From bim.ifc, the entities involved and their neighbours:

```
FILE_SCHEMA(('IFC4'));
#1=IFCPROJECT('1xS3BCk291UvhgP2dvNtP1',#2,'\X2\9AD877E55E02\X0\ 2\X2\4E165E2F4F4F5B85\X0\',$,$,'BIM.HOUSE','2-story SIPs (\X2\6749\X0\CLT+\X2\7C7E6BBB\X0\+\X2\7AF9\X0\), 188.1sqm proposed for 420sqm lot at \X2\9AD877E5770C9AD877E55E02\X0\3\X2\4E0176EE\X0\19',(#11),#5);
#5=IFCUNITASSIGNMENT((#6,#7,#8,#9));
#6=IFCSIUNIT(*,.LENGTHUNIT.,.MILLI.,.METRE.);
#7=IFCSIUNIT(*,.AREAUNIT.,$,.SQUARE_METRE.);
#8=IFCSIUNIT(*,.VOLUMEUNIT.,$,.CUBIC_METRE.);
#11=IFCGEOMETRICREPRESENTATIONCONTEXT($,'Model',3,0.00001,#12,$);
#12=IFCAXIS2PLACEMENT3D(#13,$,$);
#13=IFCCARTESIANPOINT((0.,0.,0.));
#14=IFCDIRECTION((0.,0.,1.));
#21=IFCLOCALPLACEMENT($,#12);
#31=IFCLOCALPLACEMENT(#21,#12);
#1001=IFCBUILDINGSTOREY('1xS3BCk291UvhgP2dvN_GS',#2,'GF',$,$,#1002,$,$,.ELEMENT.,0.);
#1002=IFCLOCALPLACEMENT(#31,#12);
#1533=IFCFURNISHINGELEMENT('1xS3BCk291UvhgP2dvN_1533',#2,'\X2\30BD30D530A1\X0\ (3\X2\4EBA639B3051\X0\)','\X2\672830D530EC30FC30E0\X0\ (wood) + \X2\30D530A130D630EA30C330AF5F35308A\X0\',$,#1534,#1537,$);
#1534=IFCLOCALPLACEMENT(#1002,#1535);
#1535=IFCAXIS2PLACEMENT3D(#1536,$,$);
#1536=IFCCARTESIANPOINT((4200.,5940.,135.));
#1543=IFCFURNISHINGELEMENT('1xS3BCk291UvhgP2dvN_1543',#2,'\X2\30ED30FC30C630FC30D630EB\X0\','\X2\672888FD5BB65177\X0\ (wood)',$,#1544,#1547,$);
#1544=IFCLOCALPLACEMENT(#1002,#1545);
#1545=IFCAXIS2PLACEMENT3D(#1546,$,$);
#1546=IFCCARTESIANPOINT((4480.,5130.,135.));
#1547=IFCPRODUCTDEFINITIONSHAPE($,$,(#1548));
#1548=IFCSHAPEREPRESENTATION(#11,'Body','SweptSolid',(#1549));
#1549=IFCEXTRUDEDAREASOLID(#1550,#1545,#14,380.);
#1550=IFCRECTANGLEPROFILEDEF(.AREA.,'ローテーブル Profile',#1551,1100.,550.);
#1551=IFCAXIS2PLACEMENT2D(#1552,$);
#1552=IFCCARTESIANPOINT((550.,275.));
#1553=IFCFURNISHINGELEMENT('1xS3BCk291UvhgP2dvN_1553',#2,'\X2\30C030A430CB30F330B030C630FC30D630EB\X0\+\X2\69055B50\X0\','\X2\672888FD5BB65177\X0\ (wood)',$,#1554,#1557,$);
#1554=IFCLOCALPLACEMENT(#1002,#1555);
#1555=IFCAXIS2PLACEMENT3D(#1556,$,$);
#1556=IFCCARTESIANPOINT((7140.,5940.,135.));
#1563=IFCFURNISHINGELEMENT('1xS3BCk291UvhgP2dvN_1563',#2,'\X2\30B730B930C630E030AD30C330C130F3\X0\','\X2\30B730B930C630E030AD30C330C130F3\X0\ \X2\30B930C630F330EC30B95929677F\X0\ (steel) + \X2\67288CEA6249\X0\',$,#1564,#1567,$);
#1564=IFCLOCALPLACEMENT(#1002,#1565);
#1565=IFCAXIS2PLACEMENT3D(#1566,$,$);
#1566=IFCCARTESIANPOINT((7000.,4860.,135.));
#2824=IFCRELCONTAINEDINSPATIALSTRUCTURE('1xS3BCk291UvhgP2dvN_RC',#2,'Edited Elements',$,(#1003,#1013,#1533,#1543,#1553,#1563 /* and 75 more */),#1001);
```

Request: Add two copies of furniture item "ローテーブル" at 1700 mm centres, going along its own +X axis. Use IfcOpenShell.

```python
import ifcopenshell
import ifcopenshell.api.geometry
import ifcopenshell.api.root
import ifcopenshell.util.element
import ifcopenshell.util.placement
import ifcopenshell.util.unit

model = ifcopenshell.open("bim.ifc")
unit_scale = ifcopenshell.util.unit.calculate_unit_scale(model)


def reuse_history(source, copy):
    """copy_class also copies each property set's owner history, people and application; keep the originals."""
    for rel in copy.IsDefinedBy:
        if rel.is_a("IfcRelDefinesByProperties") and (history := rel.RelatingPropertyDefinition.OwnerHistory):
            rel.RelatingPropertyDefinition.OwnerHistory = source.OwnerHistory
            ifcopenshell.util.element.remove_deep2(model, history)


source = model.by_id(1543)
base = ifcopenshell.util.placement.get_local_placement(source.ObjectPlacement)
step = base[:3, 0] * 1.7 / unit_scale

for i in range(1, 3):
    copy = ifcopenshell.api.root.copy_class(model, product=source)
    copy.Representation = ifcopenshell.util.element.copy_deep(
        model, source.Representation, exclude=["IfcGeometricRepresentationContext", "IfcRepresentationMap"]
    )
    reuse_history(source, copy)
    matrix = base.copy()
    matrix[:3, 3] += i * step
    print("added at", matrix[:3, 3].round(3) + 0.0)
    ifcopenshell.api.geometry.edit_object_placement(model, product=copy, matrix=matrix, is_si=False)

model.write("bim_updated.ifc")
```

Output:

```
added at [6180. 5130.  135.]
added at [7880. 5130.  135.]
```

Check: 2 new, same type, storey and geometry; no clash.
